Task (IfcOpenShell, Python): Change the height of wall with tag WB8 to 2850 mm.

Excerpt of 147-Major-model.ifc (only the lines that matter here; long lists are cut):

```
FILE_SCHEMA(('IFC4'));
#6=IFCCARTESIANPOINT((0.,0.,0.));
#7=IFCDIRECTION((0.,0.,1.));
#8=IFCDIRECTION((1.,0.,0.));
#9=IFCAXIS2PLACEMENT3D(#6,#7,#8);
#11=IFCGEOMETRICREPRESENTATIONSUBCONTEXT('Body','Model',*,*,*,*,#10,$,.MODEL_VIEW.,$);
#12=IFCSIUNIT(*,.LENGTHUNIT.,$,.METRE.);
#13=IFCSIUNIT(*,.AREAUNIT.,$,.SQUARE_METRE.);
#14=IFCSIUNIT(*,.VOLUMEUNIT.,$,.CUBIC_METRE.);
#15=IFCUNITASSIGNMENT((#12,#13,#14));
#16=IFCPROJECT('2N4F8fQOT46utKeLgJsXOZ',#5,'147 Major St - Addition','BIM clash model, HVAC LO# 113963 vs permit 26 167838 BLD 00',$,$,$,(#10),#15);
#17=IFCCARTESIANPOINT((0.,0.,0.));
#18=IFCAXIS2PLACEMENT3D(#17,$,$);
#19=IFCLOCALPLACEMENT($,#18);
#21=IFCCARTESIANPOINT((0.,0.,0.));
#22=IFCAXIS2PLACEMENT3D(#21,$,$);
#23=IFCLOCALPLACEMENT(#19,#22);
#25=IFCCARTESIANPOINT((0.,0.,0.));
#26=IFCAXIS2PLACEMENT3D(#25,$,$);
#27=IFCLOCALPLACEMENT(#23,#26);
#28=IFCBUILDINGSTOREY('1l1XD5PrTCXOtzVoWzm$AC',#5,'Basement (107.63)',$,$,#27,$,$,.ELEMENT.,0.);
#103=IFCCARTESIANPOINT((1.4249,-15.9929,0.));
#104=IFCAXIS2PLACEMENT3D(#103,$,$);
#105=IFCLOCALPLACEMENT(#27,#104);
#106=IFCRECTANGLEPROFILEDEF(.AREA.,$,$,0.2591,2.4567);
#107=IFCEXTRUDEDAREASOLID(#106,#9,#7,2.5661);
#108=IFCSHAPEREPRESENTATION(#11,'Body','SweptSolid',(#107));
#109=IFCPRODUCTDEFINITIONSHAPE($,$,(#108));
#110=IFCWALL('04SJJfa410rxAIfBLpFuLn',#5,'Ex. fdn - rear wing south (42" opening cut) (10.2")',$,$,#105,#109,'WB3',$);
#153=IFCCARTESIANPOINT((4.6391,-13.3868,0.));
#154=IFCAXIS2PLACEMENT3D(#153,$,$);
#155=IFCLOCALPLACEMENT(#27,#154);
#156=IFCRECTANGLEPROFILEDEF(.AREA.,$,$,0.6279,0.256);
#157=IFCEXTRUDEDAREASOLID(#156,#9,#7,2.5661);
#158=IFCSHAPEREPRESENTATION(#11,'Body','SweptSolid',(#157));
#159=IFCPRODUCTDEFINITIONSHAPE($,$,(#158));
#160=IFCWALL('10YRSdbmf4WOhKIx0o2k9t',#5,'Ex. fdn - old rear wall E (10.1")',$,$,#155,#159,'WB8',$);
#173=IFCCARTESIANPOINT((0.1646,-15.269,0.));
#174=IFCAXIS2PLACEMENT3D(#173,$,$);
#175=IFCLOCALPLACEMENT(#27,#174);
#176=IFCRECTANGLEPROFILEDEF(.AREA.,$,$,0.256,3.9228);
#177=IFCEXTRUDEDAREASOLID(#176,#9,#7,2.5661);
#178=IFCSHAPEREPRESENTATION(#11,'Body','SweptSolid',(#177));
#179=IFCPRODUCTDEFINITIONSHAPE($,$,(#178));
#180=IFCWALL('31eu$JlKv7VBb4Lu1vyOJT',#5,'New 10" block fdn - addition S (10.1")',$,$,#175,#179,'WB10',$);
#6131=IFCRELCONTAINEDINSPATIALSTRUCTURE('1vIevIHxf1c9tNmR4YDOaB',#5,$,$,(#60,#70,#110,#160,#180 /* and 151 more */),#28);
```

```python
import ifcopenshell
import ifcopenshell.geom
import ifcopenshell.util.representation
import ifcopenshell.util.shape
import ifcopenshell.util.unit

model = ifcopenshell.open("147-Major-model.ifc")
unit_scale = ifcopenshell.util.unit.calculate_unit_scale(model)
settings = ifcopenshell.geom.settings()


def volume(element):
    """Net volume in cubic metres, openings subtracted."""
    shape = ifcopenshell.geom.create_shape(settings, element)
    return ifcopenshell.util.shape.get_volume(shape.geometry)


wall = model.by_id(160)
before = volume(wall)

body = ifcopenshell.util.representation.get_representation(wall, "Model", "Body")
solid = body.Items[0]
old_height = solid.Depth
solid.Depth = 2.85 / unit_scale
after = volume(wall)

print(f"height {old_height:g} -> {solid.Depth:g}, volume {before:.3f} -> {after:.3f} m3")

model.write("147-Major-model_edited.ifc")
```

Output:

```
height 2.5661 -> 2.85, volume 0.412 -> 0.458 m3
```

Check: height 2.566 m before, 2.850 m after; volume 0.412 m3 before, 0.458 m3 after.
